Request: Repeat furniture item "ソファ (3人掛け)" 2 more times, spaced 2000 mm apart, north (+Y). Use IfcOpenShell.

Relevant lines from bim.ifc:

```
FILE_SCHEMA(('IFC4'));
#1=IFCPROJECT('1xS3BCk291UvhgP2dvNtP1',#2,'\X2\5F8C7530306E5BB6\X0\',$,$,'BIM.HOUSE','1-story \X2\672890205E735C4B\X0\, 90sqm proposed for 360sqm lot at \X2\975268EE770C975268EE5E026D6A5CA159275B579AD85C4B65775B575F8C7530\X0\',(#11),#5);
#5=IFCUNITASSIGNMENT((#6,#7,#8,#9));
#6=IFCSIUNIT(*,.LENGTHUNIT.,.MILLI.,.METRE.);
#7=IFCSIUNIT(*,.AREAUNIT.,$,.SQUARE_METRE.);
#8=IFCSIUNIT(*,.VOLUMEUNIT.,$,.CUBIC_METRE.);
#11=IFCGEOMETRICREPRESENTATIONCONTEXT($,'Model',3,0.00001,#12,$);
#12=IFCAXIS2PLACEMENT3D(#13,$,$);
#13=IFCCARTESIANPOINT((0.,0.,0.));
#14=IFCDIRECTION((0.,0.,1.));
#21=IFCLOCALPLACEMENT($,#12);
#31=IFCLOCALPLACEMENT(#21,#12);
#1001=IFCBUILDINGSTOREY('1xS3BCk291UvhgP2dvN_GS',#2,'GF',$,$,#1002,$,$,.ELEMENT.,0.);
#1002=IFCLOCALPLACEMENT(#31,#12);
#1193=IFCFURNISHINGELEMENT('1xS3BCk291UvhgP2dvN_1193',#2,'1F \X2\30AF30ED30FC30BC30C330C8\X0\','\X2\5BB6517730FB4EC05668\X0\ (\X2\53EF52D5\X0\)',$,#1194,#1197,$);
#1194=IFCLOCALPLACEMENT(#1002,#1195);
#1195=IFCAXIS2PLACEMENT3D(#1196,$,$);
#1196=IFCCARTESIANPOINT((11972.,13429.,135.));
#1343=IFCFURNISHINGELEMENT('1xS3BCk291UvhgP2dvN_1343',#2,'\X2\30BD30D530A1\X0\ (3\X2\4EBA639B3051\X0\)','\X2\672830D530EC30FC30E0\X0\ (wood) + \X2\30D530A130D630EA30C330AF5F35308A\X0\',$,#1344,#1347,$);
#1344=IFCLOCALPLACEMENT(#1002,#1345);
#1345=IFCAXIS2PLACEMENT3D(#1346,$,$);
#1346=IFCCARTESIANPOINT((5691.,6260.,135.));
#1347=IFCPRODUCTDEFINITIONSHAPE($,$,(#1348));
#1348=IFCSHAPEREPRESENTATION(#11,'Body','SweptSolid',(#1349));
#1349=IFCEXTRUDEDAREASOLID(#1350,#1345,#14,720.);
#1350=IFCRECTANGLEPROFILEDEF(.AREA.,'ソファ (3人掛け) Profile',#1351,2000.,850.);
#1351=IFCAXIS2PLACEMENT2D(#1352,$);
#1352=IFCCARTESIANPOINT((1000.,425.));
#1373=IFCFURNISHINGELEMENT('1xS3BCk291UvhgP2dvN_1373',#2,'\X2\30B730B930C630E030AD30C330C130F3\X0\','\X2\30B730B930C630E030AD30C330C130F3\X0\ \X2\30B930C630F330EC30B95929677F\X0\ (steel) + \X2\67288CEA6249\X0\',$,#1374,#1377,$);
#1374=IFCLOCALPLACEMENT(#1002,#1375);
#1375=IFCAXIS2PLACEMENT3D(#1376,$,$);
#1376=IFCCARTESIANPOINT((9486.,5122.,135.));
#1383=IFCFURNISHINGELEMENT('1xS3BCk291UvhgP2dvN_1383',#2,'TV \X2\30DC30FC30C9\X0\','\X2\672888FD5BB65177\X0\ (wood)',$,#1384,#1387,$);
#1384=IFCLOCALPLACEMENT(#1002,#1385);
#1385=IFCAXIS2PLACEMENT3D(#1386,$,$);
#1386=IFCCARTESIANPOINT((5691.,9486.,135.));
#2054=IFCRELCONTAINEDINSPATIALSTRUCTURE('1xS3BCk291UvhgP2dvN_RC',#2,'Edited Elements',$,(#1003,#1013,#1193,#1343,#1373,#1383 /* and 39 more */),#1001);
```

```python
import numpy as np
import ifcopenshell
import ifcopenshell.api.geometry
import ifcopenshell.api.root
import ifcopenshell.util.element
import ifcopenshell.util.placement
import ifcopenshell.util.unit

model = ifcopenshell.open("bim.ifc")
unit_scale = ifcopenshell.util.unit.calculate_unit_scale(model)


def reuse_history(source, copy):
    """copy_class also copies each property set's owner history, people and application; keep the originals."""
    for rel in copy.IsDefinedBy:
        if rel.is_a("IfcRelDefinesByProperties") and (history := rel.RelatingPropertyDefinition.OwnerHistory):
            rel.RelatingPropertyDefinition.OwnerHistory = source.OwnerHistory
            ifcopenshell.util.element.remove_deep2(model, history)


source = model.by_guid("1xS3BCk291UvhgP2dvN_1343")
base = ifcopenshell.util.placement.get_local_placement(source.ObjectPlacement)
step = np.array([0.0, 1.0, 0.0]) * 2 / unit_scale

for i in range(1, 3):
    copy = ifcopenshell.api.root.copy_class(model, product=source)
    copy.Representation = ifcopenshell.util.element.copy_deep(
        model, source.Representation, exclude=["IfcGeometricRepresentationContext", "IfcRepresentationMap"]
    )
    reuse_history(source, copy)
    matrix = base.copy()
    matrix[:3, 3] += i * step
    print("added at", matrix[:3, 3].round(3) + 0.0)
    ifcopenshell.api.geometry.edit_object_placement(model, product=copy, matrix=matrix, is_si=False)

model.write("bim_rev.ifc")
```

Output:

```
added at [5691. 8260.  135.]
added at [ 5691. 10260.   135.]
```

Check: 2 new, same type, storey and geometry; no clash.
